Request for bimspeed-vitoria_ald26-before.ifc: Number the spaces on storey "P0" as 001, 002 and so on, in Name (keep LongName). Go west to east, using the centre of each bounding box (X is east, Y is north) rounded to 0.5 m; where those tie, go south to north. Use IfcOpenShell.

First a look at what the model holds.

```python
import ifcopenshell
import ifcopenshell.util.element
import ifcopenshell.util.placement

model = ifcopenshell.open("bimspeed-vitoria_ald26-before.ifc")
print(model.schema)
storey = next(s for s in model.by_type("IfcBuildingStorey") if s.Name == "P0")
spaces = [e for e in ifcopenshell.util.element.get_decomposition(storey) if e.is_a("IfcSpace")]
for e in sorted(spaces, key=lambda e: e.id()):
    origin = ifcopenshell.util.placement.get_local_placement(e.ObjectPlacement)[:3, 3]
    print(e.id(), e.Name, e.LongName, origin.round(2) + 0.0, sep=" | ")
```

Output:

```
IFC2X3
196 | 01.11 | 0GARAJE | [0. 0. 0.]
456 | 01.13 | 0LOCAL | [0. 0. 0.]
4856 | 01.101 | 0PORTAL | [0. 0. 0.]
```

```python
import ifcopenshell
import ifcopenshell.geom
import ifcopenshell.util.element
import ifcopenshell.util.shape

model = ifcopenshell.open("bimspeed-vitoria_ald26-before.ifc")
settings = ifcopenshell.geom.settings()
settings.set("use-world-coords", True)


def centre(element):
    shape = ifcopenshell.geom.create_shape(settings, element)
    return ifcopenshell.util.shape.get_bbox_centroid(shape.geometry)


storey = next(s for s in model.by_type("IfcBuildingStorey") if s.Name == "P0")
spaces = [e for e in ifcopenshell.util.element.get_decomposition(storey) if e.is_a("IfcSpace")]

# Insertion points can sit at a corner or the storey origin, so sort by the geometry (in metres).
centres = {e: centre(e) for e in spaces}
spaces.sort(key=lambda e: (round(centres[e][0] / 0.5), centres[e][1]))

for i, e in enumerate(spaces, start=1):
    number = f"0{i:02d}"
    e.Name = number
    print(e.id(), number)

model.write("bimspeed-vitoria_ald26-before-out.ifc")
```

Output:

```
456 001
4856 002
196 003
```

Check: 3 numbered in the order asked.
